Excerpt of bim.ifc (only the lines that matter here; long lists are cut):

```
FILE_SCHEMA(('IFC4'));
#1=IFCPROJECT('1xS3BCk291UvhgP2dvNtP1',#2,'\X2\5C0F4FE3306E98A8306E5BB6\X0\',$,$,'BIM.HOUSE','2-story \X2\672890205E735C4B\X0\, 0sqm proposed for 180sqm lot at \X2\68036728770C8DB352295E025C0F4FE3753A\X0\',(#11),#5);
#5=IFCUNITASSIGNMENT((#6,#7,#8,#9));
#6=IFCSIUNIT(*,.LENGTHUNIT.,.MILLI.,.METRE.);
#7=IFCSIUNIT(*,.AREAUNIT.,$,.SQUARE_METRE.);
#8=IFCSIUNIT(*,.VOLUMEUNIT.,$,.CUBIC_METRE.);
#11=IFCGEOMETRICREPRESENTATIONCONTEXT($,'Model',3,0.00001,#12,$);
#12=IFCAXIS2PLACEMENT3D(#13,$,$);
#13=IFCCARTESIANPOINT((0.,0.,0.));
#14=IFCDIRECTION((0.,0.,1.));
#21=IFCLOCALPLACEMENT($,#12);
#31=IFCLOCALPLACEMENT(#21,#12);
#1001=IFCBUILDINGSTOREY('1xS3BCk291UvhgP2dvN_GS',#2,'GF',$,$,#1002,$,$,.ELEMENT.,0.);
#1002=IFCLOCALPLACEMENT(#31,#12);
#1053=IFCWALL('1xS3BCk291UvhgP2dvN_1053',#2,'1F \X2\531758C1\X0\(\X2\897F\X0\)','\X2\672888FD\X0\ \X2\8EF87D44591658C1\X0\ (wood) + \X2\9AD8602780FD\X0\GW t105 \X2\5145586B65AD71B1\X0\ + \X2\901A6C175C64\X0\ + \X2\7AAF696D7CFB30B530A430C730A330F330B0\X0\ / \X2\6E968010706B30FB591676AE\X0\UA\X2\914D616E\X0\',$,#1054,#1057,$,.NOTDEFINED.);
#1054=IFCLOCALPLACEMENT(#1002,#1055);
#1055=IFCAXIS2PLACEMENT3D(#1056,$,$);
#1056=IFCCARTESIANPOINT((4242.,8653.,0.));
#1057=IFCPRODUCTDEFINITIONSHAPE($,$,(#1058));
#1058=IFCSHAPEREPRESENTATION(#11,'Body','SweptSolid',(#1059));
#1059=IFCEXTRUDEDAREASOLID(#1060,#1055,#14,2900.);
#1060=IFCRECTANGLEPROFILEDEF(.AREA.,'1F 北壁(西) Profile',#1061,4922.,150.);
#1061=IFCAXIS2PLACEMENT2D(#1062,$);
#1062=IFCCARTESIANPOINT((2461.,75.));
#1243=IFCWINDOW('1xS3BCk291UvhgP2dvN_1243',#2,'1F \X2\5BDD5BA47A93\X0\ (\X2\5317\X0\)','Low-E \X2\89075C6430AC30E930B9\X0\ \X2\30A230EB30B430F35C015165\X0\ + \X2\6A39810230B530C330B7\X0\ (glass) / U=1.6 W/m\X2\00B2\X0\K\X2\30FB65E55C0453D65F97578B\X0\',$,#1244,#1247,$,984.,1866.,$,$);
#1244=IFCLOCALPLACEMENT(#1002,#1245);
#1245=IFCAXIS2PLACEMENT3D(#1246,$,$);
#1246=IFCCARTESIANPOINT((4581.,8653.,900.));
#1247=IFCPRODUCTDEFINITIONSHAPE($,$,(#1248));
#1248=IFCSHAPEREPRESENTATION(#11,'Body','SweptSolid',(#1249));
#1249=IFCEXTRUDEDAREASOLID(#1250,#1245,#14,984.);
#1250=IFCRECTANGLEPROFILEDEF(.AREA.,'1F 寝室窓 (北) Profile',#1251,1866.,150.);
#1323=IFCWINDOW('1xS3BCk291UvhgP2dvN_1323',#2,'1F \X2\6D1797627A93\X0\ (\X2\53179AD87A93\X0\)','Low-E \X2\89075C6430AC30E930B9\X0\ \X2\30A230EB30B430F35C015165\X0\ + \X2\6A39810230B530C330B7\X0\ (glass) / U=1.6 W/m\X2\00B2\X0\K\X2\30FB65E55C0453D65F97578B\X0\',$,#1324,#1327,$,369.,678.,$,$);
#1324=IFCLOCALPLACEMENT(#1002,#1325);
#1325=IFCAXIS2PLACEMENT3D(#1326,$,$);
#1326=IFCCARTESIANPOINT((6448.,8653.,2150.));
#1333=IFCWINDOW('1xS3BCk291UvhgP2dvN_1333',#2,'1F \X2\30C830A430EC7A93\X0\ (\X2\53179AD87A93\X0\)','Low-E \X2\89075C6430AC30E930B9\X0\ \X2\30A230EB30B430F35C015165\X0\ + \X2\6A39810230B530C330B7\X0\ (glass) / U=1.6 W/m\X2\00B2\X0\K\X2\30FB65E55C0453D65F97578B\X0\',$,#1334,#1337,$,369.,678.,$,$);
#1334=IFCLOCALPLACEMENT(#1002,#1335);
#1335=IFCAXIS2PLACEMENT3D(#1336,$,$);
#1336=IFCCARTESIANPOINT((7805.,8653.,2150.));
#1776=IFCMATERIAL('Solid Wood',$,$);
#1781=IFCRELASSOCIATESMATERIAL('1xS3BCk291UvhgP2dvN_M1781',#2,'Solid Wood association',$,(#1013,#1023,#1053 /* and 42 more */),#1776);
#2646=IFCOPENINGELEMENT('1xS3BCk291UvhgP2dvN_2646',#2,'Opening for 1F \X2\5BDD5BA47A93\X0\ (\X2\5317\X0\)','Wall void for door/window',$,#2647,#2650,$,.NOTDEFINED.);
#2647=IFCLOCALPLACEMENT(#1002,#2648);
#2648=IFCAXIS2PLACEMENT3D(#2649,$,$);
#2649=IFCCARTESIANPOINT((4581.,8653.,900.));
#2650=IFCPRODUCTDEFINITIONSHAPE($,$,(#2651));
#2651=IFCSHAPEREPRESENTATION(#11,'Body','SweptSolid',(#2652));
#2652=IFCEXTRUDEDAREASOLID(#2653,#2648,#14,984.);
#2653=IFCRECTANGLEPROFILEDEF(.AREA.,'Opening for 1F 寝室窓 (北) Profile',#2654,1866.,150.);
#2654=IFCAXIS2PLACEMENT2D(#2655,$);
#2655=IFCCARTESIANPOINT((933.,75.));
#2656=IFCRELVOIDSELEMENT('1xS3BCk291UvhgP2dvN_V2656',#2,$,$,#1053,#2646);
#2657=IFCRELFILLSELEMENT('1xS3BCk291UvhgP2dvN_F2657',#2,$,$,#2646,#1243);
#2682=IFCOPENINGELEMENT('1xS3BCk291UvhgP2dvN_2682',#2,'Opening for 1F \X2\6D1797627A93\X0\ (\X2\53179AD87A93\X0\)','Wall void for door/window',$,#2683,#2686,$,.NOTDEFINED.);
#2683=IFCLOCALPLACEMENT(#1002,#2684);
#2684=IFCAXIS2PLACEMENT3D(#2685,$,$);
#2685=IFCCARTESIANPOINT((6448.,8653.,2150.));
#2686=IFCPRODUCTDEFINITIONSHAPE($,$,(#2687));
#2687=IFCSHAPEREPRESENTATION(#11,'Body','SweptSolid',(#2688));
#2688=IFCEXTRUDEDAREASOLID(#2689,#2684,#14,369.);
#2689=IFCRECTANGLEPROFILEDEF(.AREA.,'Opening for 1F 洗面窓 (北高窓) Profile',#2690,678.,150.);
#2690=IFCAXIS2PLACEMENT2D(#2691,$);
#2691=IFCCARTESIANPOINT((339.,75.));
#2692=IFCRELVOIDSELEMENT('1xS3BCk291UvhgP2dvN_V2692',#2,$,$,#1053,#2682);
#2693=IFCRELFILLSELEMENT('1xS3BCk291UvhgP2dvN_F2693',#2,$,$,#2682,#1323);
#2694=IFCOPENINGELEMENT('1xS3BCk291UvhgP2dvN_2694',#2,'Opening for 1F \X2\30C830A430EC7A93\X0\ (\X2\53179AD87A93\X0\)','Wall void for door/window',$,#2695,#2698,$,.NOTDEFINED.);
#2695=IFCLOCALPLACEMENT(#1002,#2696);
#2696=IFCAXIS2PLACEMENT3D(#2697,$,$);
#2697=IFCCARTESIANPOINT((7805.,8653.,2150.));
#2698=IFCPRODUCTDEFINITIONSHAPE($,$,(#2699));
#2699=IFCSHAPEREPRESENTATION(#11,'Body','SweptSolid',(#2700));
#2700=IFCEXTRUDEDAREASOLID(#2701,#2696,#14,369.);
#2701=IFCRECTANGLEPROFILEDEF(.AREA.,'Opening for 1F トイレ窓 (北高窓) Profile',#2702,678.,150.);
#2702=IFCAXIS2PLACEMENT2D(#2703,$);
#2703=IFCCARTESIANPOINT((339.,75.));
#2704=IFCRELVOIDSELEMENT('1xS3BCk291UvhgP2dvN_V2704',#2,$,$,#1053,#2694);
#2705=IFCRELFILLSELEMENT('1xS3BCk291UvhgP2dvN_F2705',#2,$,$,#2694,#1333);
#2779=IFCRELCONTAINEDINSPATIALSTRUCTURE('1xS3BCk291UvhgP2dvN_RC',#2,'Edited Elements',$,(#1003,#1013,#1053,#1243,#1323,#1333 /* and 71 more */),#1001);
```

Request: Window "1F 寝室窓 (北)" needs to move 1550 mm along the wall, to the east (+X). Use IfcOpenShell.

```python
import ifcopenshell
import ifcopenshell.api.geometry
import ifcopenshell.util.placement
import ifcopenshell.util.unit

model = ifcopenshell.open("bim.ifc")
unit_scale = ifcopenshell.util.unit.calculate_unit_scale(model)

window = model.by_guid("1xS3BCk291UvhgP2dvN_1243")
opening = window.FillsVoids[0].RelatingOpeningElement
wall = opening.VoidsElements[0].RelatingBuildingElement

wall_matrix = ifcopenshell.util.placement.get_local_placement(wall.ObjectPlacement)
shift = wall_matrix[:3, 0] * 1.55 / unit_scale
before = ifcopenshell.util.placement.get_local_placement(window.ObjectPlacement)[:3, 3].copy()

# The window is not placed relative to its opening, so move both.
for product in (opening, window):
    matrix = ifcopenshell.util.placement.get_local_placement(product.ObjectPlacement)
    matrix[:3, 3] += shift
    ifcopenshell.api.geometry.edit_object_placement(model, product=product, matrix=matrix, is_si=False)

after = ifcopenshell.util.placement.get_local_placement(window.ObjectPlacement)[:3, 3]
print("window moved by", (after - before).round(3) + 0.0)

model.write("bim_rev.ifc")
```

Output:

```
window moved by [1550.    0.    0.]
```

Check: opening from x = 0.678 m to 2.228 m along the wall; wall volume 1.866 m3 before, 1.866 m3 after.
